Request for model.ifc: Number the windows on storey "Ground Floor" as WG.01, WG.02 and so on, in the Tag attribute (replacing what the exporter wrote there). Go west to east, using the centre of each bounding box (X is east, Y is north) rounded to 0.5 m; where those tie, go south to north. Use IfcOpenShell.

First a look at what the model holds.

```python
import ifcopenshell
import ifcopenshell.util.element
import ifcopenshell.util.placement

model = ifcopenshell.open("model.ifc")
print(model.schema)
storey = next(s for s in model.by_type("IfcBuildingStorey") if s.Name == "Ground Floor")
windows = [e for e in ifcopenshell.util.element.get_decomposition(storey) if e.is_a("IfcWindow")]
for e in sorted(windows, key=lambda e: e.id()):
    origin = ifcopenshell.util.placement.get_local_placement(e.ObjectPlacement)[:3, 3]
    print(e.id(), e.Tag, e.Name, origin.round(2) + 0.0, sep=" | ")
```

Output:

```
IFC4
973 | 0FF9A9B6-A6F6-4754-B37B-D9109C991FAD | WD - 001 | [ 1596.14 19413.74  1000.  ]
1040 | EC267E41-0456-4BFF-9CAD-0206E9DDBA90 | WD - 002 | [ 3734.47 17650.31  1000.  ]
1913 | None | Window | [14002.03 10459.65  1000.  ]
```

```python
import ifcopenshell
import ifcopenshell.geom
import ifcopenshell.util.element
import ifcopenshell.util.shape

model = ifcopenshell.open("model.ifc")
settings = ifcopenshell.geom.settings()
settings.set("use-world-coords", True)


def centre(element):
    shape = ifcopenshell.geom.create_shape(settings, element)
    return ifcopenshell.util.shape.get_bbox_centroid(shape.geometry)


storey = next(s for s in model.by_type("IfcBuildingStorey") if s.Name == "Ground Floor")
windows = [e for e in ifcopenshell.util.element.get_decomposition(storey) if e.is_a("IfcWindow")]

# Insertion points can sit at a corner or the storey origin, so sort by the geometry (in metres).
centres = {e: centre(e) for e in windows}
windows.sort(key=lambda e: (round(centres[e][0] / 0.5), centres[e][1]))

for i, e in enumerate(windows, start=1):
    number = f"WG.{i:02d}"
    e.Tag = number
    print(e.id(), number)

model.write("model_v2.ifc")
```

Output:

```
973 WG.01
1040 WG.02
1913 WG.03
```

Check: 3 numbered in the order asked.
